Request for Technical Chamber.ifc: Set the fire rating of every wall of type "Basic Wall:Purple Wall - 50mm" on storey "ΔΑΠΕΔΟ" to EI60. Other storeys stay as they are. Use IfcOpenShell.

First a look at what the model holds.

```python
import ifcopenshell
import ifcopenshell.util.element

model = ifcopenshell.open("Technical Chamber.ifc")
print(model.schema)
storey = next(s for s in model.by_type("IfcBuildingStorey") if s.Name == "ΔΑΠΕΔΟ")
walls = [e for e in ifcopenshell.util.element.get_decomposition(storey) if e.is_a("IfcWall")]
seen = {}
for e in walls:
    element_type = ifcopenshell.util.element.get_type(e)
    key = (element_type.Name if element_type != e and element_type else None, ifcopenshell.util.element.get_pset(e, "Pset_WallCommon", "FireRating"))
    seen[key] = seen.get(key, 0) + 1
for (name, value), count in sorted(seen.items(), key=str):
    print(count, "x", name, "|", value)
```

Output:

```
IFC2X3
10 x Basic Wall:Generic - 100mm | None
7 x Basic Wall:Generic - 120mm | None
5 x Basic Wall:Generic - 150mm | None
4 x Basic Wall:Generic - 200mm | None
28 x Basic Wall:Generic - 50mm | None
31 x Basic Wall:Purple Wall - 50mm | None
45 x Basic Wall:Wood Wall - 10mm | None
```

```python
import ifcopenshell
import ifcopenshell.api.pset
import ifcopenshell.util.element

model = ifcopenshell.open("Technical Chamber.ifc")

storey = next(s for s in model.by_type("IfcBuildingStorey") if s.Name == "ΔΑΠΕΔΟ")
walls = [e for e in ifcopenshell.util.element.get_decomposition(storey) if e.is_a("IfcWall")]

count = 0
for e in walls:
    element_type = ifcopenshell.util.element.get_type(e)
    if element_type in (None, e) or element_type.Name != "Basic Wall:Purple Wall - 50mm":
        continue
    # add_pset returns the element's existing set when there is one.
    pset = ifcopenshell.api.pset.add_pset(model, product=e, name="Pset_WallCommon")
    ifcopenshell.api.pset.edit_pset(model, pset=pset, properties={"FireRating": "EI60"})
    count += 1

print(count, "walls updated")

model.write("Technical Chamber-out.ifc")
```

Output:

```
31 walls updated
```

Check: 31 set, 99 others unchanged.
